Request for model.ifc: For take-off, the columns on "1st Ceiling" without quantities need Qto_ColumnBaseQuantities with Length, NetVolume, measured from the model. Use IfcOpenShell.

First a look at what the model holds.

```python
import ifcopenshell
import ifcopenshell.util.element
import ifcopenshell.util.unit

model = ifcopenshell.open("model.ifc")
print(model.schema)
for unit_type in ("LENGTHUNIT", "AREAUNIT", "VOLUMEUNIT"):
    print(unit_type, ifcopenshell.util.unit.calculate_unit_scale(model, unit_type))
storey = next(s for s in model.by_type("IfcBuildingStorey") if s.Name == "1st Ceiling")
columns = [e for e in ifcopenshell.util.element.get_decomposition(storey) if e.is_a("IfcColumn")]
for e in sorted(columns, key=lambda e: e.id()):
    print(e.id(), e.is_a(), e.Name, list(ifcopenshell.util.element.get_psets(e, qtos_only=True)), sep=" | ")
```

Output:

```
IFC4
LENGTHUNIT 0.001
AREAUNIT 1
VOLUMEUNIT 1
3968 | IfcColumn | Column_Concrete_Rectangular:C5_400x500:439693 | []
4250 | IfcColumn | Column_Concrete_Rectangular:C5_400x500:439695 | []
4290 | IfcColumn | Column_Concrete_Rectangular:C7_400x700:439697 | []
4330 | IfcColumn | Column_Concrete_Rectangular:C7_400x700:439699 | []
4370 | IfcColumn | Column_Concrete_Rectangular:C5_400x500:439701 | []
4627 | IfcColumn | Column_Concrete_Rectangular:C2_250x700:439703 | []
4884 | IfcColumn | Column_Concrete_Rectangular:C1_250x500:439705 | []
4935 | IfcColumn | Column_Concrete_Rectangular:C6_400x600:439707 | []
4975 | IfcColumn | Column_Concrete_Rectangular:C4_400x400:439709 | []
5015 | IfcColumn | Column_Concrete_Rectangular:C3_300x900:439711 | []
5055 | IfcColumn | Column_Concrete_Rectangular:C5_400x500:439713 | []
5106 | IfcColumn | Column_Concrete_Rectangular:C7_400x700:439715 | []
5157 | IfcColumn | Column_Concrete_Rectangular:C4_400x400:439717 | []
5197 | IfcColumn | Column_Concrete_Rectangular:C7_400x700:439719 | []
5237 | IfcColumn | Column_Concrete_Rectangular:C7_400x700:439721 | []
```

```python
import ifcopenshell
import ifcopenshell.api.pset
import ifcopenshell.geom
import ifcopenshell.util.element
import ifcopenshell.util.shape
import ifcopenshell.util.unit

model = ifcopenshell.open("model.ifc")
unit_scale = ifcopenshell.util.unit.calculate_unit_scale(model)
volume_scale = ifcopenshell.util.unit.calculate_unit_scale(model, "VOLUMEUNIT")
settings = ifcopenshell.geom.settings()

storey = next(s for s in model.by_type("IfcBuildingStorey") if s.Name == "1st Ceiling")
columns = [e for e in ifcopenshell.util.element.get_decomposition(storey) if e.is_a("IfcColumn")]

for e in sorted(columns, key=lambda e: e.id()):
    if ifcopenshell.util.element.get_psets(e, qtos_only=True, should_inherit=False):
        continue
    # Geometry comes back in metres, in the element's own axes.
    shape = ifcopenshell.geom.create_shape(settings, e)
    values = {
        "Length": ifcopenshell.util.shape.get_z(shape.geometry) / unit_scale,
        "NetVolume": ifcopenshell.util.shape.get_volume(shape.geometry) / volume_scale,
    }
    qto = ifcopenshell.api.pset.add_qto(model, product=e, name="Qto_ColumnBaseQuantities")
    ifcopenshell.api.pset.edit_qto(model, qto=qto, properties=values)
    print(e.id(), {k: round(v, 3) for k, v in values.items()})

model.write("model_edited.ifc")
```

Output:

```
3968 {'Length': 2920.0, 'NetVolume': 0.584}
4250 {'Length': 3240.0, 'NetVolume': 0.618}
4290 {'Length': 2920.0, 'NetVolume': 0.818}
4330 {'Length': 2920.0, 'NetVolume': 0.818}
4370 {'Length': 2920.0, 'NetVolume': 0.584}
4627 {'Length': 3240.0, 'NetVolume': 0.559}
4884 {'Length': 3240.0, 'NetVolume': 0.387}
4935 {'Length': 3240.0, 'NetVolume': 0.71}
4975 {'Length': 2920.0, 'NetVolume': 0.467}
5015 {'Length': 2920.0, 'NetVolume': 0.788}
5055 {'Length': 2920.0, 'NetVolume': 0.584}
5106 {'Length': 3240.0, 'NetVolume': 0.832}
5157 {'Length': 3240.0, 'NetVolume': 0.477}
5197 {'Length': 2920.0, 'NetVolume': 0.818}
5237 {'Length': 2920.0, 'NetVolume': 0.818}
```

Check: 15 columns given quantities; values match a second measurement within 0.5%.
